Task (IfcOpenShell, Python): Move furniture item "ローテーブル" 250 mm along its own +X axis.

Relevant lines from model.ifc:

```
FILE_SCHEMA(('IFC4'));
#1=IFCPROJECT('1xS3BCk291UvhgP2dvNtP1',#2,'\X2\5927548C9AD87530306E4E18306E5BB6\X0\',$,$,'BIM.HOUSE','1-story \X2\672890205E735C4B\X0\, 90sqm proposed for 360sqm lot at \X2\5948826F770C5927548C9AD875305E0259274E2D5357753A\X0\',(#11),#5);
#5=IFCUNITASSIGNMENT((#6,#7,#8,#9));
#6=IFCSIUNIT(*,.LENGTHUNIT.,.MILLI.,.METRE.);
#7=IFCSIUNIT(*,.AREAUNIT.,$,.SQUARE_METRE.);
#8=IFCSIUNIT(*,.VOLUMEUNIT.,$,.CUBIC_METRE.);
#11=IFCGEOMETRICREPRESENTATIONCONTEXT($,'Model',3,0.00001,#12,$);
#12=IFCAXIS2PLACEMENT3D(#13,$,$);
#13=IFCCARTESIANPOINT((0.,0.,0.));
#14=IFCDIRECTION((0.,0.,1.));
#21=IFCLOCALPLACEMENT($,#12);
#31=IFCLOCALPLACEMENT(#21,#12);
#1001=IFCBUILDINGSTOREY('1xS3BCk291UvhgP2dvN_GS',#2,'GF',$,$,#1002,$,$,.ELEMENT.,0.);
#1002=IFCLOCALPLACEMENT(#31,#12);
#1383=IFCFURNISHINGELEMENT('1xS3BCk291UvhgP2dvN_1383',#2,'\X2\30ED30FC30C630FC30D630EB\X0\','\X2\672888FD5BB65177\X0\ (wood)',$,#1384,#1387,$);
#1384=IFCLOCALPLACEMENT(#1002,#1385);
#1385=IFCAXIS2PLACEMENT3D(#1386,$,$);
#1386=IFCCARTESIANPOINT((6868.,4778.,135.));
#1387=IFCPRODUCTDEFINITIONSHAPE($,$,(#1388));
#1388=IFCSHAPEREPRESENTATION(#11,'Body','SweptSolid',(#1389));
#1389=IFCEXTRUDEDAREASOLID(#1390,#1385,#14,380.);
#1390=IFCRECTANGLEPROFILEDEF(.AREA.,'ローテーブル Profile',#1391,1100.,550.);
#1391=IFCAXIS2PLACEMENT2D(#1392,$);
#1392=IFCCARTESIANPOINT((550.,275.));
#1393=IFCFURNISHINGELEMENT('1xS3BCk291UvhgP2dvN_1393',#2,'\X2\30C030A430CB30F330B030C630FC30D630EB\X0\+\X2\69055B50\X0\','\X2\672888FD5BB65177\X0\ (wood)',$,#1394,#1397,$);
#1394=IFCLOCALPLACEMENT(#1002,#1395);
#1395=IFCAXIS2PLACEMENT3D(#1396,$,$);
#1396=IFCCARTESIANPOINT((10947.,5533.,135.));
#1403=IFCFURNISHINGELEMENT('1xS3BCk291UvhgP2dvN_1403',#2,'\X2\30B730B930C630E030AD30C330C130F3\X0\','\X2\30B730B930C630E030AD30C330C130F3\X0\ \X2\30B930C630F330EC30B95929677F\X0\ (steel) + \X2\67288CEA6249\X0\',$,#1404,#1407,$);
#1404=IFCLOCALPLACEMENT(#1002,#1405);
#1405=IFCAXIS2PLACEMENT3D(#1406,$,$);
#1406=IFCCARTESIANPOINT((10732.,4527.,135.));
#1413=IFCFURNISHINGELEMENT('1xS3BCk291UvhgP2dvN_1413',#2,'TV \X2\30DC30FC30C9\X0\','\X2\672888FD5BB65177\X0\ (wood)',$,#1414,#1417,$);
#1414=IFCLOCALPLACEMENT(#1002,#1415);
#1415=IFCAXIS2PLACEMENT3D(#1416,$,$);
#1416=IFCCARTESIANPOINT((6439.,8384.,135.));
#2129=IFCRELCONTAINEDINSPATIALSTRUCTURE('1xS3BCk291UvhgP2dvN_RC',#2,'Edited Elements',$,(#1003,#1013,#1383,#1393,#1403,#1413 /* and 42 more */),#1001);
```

```python
import ifcopenshell
import ifcopenshell.api.geometry
import ifcopenshell.util.placement

model = ifcopenshell.open("model.ifc")

item = model.by_guid("1xS3BCk291UvhgP2dvN_1383")
matrix = ifcopenshell.util.placement.get_local_placement(item.ObjectPlacement)
matrix[:3, 3] += matrix[:3, 0] * 250.0
ifcopenshell.api.geometry.edit_object_placement(model, product=item, matrix=matrix, is_si=False)

print(ifcopenshell.util.placement.get_local_placement(item.ObjectPlacement).round(3) + 0.0)

model.write("model_rev.ifc")
```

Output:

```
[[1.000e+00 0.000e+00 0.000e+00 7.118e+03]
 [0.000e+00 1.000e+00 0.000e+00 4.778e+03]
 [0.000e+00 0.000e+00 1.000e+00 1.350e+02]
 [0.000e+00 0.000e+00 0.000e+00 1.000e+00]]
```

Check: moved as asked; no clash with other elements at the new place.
